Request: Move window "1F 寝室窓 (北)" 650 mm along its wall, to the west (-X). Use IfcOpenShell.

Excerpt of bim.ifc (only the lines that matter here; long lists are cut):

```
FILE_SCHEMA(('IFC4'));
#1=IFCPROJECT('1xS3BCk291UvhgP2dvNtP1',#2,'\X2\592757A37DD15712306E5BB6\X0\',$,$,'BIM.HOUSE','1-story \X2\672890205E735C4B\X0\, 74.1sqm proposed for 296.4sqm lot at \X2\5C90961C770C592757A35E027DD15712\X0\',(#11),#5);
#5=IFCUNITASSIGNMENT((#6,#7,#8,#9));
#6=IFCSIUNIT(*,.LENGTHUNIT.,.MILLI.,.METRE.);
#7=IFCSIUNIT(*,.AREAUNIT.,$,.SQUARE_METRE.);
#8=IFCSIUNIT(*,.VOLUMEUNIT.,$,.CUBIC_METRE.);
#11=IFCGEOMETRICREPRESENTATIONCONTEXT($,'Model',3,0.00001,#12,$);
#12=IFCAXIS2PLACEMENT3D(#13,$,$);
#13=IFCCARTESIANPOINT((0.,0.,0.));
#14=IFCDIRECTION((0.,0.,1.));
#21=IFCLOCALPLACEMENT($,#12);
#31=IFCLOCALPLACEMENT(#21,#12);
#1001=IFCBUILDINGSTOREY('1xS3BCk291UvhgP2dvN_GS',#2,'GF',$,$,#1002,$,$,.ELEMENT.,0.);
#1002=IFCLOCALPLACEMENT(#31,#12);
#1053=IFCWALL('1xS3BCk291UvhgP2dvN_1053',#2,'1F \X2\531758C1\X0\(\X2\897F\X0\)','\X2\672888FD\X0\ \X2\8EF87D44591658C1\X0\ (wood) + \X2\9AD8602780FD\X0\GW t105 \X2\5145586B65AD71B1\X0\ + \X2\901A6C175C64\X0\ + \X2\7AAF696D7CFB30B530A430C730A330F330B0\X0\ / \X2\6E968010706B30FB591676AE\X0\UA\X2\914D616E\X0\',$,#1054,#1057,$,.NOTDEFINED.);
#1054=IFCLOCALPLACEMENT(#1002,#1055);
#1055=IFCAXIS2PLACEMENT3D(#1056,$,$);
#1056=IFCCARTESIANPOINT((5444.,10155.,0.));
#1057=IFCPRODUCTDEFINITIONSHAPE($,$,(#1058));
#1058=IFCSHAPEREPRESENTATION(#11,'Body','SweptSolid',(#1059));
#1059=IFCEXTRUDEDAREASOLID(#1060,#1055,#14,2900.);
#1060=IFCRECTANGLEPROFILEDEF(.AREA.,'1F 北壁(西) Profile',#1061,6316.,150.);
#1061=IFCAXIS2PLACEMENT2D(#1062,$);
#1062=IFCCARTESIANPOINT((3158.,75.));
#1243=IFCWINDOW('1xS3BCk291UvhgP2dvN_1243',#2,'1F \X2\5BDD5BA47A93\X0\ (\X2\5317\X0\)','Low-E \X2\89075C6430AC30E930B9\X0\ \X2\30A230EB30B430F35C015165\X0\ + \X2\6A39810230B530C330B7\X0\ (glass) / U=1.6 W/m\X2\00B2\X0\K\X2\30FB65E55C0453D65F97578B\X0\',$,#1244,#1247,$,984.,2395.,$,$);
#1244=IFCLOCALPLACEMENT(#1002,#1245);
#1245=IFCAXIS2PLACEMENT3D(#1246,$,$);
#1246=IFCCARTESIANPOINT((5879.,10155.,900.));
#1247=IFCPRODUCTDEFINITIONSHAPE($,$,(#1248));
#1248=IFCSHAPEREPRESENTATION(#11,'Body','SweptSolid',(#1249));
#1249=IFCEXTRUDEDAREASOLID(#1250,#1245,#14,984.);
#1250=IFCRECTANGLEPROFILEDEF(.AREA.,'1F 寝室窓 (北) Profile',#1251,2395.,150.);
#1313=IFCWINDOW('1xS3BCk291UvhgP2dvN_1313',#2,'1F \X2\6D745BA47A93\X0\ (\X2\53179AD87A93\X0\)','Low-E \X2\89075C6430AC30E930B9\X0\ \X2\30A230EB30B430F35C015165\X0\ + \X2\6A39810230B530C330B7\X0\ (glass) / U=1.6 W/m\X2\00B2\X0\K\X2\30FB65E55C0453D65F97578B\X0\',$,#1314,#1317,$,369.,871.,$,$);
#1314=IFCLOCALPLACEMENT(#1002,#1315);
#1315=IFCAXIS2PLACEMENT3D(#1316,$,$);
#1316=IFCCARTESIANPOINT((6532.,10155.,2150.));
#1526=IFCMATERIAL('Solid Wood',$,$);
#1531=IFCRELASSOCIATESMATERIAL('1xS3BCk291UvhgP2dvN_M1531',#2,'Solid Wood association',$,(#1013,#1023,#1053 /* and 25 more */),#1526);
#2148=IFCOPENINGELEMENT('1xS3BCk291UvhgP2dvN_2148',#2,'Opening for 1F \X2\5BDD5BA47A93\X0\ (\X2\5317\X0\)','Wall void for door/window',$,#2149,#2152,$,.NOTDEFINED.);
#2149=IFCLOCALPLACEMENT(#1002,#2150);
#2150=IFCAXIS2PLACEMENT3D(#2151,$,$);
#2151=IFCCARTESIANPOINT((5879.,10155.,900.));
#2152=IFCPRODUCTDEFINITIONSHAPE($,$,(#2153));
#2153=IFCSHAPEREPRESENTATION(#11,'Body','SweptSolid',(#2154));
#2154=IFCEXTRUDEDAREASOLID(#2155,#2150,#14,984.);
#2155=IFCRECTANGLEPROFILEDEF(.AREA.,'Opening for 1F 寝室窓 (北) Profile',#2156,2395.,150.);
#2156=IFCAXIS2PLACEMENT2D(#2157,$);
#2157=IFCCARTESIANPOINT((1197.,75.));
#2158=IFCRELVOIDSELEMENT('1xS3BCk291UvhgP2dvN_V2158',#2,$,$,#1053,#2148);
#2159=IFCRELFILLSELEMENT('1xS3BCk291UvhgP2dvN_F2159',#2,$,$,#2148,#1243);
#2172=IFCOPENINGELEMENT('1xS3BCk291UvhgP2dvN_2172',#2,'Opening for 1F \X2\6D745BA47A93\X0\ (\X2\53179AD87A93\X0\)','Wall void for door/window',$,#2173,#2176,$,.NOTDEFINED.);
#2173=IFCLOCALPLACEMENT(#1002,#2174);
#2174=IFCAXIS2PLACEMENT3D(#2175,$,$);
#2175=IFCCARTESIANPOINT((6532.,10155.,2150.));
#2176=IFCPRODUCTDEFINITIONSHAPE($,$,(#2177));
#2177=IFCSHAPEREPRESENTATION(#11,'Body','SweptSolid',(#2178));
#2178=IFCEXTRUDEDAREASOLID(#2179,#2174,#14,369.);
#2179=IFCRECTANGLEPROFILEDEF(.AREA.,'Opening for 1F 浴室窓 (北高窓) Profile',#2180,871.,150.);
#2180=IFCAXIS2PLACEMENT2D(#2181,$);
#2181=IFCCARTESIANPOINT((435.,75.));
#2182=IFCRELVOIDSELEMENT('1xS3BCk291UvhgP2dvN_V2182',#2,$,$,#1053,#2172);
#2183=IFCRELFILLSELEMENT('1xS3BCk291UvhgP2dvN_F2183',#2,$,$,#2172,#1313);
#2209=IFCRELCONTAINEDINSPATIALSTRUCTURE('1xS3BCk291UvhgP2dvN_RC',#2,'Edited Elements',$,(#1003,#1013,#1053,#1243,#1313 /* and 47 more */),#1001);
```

```python
import ifcopenshell
import ifcopenshell.api.geometry
import ifcopenshell.util.placement
import ifcopenshell.util.unit

model = ifcopenshell.open("bim.ifc")
unit_scale = ifcopenshell.util.unit.calculate_unit_scale(model)

window = model.by_guid("1xS3BCk291UvhgP2dvN_1243")
opening = window.FillsVoids[0].RelatingOpeningElement
wall = opening.VoidsElements[0].RelatingBuildingElement

wall_matrix = ifcopenshell.util.placement.get_local_placement(wall.ObjectPlacement)
shift = wall_matrix[:3, 0] * -0.65 / unit_scale
before = ifcopenshell.util.placement.get_local_placement(window.ObjectPlacement)[:3, 3].copy()

# The window is not placed relative to its opening, so move both.
for product in (opening, window):
    matrix = ifcopenshell.util.placement.get_local_placement(product.ObjectPlacement)
    matrix[:3, 3] += shift
    ifcopenshell.api.geometry.edit_object_placement(model, product=product, matrix=matrix, is_si=False)

after = ifcopenshell.util.placement.get_local_placement(window.ObjectPlacement)[:3, 3]
print("window moved by", (after - before).round(3) + 0.0)

model.write("bim_updated.ifc")
```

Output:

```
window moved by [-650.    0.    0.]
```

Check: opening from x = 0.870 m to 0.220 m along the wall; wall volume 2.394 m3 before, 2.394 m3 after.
